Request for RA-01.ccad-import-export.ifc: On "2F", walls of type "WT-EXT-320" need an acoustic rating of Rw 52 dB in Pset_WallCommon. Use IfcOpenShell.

First a look at what the model holds.

```python
import ifcopenshell
import ifcopenshell.util.element

model = ifcopenshell.open("RA-01.ccad-import-export.ifc")
print(model.schema)
storey = next(s for s in model.by_type("IfcBuildingStorey") if s.Name == "2F")
walls = [e for e in ifcopenshell.util.element.get_decomposition(storey) if e.is_a("IfcWall")]
seen = {}
for e in walls:
    element_type = ifcopenshell.util.element.get_type(e)
    key = (element_type.Name if element_type != e and element_type else None, ifcopenshell.util.element.get_pset(e, "Pset_WallCommon", "AcousticRating"))
    seen[key] = seen.get(key, 0) + 1
for (name, value), count in sorted(seen.items(), key=str):
    print(count, "x", name, "|", value)
```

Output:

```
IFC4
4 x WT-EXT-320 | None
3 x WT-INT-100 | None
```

```python
import ifcopenshell
import ifcopenshell.api.pset
import ifcopenshell.util.element

model = ifcopenshell.open("RA-01.ccad-import-export.ifc")

storey = next(s for s in model.by_type("IfcBuildingStorey") if s.Name == "2F")
walls = [e for e in ifcopenshell.util.element.get_decomposition(storey) if e.is_a("IfcWall")]

count = 0
for e in walls:
    element_type = ifcopenshell.util.element.get_type(e)
    if element_type in (None, e) or element_type.Name != "WT-EXT-320":
        continue
    # add_pset returns the element's existing set when there is one.
    pset = ifcopenshell.api.pset.add_pset(model, product=e, name="Pset_WallCommon")
    ifcopenshell.api.pset.edit_pset(model, pset=pset, properties={"AcousticRating": "Rw 52 dB"})
    count += 1

print(count, "walls updated")

model.write("RA-01.ccad-import-export_updated.ifc")
```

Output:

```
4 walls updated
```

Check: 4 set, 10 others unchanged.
